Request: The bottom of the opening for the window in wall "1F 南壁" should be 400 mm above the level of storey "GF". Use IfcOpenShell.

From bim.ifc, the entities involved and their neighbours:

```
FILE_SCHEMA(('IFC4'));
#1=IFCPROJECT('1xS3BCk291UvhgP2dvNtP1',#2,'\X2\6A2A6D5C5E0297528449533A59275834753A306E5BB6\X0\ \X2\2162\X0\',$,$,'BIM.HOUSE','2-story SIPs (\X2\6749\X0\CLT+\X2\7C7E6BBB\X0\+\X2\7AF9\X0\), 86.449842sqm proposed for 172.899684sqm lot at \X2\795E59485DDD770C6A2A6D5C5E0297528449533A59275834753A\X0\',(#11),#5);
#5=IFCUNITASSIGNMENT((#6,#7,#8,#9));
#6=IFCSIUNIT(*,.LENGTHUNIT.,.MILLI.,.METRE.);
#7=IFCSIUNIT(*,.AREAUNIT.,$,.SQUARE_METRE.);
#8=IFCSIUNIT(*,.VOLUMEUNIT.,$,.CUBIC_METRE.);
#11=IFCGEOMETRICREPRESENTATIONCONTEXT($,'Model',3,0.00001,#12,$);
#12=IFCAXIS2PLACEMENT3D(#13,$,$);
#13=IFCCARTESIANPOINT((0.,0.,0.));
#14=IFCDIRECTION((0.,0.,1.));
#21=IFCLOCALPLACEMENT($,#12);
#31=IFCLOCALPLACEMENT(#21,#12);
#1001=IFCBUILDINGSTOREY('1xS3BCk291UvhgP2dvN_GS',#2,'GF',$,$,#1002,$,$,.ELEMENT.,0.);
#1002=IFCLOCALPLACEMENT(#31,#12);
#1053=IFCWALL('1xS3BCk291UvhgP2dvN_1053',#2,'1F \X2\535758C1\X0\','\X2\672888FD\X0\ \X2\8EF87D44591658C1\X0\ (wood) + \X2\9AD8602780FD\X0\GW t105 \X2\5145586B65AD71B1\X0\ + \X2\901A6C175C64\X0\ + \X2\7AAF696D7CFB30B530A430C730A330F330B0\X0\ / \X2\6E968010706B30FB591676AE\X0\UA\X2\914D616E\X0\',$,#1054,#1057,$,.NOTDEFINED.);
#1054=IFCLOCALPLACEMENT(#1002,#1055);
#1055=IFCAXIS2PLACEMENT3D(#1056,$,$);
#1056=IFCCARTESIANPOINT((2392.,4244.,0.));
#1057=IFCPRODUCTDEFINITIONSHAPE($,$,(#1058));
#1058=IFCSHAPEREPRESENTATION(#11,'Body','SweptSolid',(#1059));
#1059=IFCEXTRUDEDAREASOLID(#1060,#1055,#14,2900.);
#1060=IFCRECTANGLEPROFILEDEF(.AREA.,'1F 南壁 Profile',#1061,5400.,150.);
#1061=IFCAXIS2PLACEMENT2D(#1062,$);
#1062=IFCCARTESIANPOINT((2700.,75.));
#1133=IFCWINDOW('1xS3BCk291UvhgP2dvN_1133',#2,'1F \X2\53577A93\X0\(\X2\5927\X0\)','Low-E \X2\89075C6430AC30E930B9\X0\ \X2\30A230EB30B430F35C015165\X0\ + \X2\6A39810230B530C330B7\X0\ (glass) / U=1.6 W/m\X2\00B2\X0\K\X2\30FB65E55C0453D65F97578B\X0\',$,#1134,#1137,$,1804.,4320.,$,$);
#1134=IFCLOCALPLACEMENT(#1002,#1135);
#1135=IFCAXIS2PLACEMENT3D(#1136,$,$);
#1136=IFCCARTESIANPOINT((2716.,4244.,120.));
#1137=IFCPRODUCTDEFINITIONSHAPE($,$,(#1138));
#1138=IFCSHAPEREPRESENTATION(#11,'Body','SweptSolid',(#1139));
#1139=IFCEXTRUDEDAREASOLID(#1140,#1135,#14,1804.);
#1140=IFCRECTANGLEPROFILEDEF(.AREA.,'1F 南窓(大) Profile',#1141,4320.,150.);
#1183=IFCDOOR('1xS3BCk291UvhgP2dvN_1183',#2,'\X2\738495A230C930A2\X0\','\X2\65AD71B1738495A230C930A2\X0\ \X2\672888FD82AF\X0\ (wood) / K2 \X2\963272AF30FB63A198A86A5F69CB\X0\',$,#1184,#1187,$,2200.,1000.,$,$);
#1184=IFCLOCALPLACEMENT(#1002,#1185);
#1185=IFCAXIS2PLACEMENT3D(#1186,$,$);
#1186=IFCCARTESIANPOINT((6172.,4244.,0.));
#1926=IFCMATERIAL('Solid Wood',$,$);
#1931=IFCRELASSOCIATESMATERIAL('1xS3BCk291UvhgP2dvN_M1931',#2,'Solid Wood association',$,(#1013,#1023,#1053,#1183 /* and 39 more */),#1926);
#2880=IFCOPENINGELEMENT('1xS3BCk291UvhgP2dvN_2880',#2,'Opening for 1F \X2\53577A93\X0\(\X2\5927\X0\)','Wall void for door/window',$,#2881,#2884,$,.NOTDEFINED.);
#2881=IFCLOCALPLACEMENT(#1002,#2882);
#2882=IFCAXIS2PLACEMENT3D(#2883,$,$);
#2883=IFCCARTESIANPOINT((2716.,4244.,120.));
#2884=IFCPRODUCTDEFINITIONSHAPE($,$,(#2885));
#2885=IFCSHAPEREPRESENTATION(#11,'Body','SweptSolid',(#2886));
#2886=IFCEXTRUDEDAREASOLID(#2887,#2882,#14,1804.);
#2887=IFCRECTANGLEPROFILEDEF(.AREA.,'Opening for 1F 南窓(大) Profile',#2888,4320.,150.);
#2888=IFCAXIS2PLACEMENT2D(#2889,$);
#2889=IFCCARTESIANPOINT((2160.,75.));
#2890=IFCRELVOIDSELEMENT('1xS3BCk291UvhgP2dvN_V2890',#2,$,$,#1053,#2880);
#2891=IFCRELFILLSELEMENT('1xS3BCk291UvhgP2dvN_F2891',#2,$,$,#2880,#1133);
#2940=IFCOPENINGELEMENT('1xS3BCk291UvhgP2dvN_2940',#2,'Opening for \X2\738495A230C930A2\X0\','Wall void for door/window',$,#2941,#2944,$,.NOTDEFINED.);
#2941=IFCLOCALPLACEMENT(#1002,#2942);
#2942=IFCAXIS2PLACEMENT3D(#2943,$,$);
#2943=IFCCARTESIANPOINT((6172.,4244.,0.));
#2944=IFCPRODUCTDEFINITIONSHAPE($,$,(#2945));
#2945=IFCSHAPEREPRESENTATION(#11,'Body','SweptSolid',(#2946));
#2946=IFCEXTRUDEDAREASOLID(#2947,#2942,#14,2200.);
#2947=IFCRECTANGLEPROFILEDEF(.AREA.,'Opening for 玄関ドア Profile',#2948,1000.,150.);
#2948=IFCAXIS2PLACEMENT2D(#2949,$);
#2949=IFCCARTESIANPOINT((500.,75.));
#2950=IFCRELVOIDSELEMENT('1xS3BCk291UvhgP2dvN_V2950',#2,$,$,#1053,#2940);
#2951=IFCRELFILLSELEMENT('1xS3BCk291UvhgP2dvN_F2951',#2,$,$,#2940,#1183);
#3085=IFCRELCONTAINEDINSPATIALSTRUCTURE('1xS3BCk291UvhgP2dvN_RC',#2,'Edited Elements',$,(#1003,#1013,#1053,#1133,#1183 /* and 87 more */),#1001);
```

```python
import numpy as np
import ifcopenshell
import ifcopenshell.api.geometry
import ifcopenshell.geom
import ifcopenshell.util.element
import ifcopenshell.util.placement
import ifcopenshell.util.shape
import ifcopenshell.util.unit

model = ifcopenshell.open("bim.ifc")
unit_scale = ifcopenshell.util.unit.calculate_unit_scale(model)

window = model.by_guid("1xS3BCk291UvhgP2dvN_1133")
opening = window.FillsVoids[0].RelatingOpeningElement
storey = ifcopenshell.util.element.get_container(window, ifc_class="IfcBuildingStorey")
level = ifcopenshell.util.placement.get_local_placement(storey.ObjectPlacement)[2, 3]

# The opening's origin need not be at the sill, so measure its lowest point.
shape = ifcopenshell.geom.create_shape(ifcopenshell.geom.settings(), opening)
bottom = ifcopenshell.util.shape.get_shape_bottom_elevation(shape, shape.geometry) / unit_scale
dz = level + 0.4 / unit_scale - bottom

shift = np.array([0.0, 0.0, dz])
# The window is not placed relative to its opening, so move both.
for product in (opening, window):
    matrix = ifcopenshell.util.placement.get_local_placement(product.ObjectPlacement)
    matrix[:3, 3] += shift
    ifcopenshell.api.geometry.edit_object_placement(model, product=product, matrix=matrix, is_si=False)

print(f"moved by {dz * unit_scale:+.3f} m")

model.write("bim-out.ifc")
```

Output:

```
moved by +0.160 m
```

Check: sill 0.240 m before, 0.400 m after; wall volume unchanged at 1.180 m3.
